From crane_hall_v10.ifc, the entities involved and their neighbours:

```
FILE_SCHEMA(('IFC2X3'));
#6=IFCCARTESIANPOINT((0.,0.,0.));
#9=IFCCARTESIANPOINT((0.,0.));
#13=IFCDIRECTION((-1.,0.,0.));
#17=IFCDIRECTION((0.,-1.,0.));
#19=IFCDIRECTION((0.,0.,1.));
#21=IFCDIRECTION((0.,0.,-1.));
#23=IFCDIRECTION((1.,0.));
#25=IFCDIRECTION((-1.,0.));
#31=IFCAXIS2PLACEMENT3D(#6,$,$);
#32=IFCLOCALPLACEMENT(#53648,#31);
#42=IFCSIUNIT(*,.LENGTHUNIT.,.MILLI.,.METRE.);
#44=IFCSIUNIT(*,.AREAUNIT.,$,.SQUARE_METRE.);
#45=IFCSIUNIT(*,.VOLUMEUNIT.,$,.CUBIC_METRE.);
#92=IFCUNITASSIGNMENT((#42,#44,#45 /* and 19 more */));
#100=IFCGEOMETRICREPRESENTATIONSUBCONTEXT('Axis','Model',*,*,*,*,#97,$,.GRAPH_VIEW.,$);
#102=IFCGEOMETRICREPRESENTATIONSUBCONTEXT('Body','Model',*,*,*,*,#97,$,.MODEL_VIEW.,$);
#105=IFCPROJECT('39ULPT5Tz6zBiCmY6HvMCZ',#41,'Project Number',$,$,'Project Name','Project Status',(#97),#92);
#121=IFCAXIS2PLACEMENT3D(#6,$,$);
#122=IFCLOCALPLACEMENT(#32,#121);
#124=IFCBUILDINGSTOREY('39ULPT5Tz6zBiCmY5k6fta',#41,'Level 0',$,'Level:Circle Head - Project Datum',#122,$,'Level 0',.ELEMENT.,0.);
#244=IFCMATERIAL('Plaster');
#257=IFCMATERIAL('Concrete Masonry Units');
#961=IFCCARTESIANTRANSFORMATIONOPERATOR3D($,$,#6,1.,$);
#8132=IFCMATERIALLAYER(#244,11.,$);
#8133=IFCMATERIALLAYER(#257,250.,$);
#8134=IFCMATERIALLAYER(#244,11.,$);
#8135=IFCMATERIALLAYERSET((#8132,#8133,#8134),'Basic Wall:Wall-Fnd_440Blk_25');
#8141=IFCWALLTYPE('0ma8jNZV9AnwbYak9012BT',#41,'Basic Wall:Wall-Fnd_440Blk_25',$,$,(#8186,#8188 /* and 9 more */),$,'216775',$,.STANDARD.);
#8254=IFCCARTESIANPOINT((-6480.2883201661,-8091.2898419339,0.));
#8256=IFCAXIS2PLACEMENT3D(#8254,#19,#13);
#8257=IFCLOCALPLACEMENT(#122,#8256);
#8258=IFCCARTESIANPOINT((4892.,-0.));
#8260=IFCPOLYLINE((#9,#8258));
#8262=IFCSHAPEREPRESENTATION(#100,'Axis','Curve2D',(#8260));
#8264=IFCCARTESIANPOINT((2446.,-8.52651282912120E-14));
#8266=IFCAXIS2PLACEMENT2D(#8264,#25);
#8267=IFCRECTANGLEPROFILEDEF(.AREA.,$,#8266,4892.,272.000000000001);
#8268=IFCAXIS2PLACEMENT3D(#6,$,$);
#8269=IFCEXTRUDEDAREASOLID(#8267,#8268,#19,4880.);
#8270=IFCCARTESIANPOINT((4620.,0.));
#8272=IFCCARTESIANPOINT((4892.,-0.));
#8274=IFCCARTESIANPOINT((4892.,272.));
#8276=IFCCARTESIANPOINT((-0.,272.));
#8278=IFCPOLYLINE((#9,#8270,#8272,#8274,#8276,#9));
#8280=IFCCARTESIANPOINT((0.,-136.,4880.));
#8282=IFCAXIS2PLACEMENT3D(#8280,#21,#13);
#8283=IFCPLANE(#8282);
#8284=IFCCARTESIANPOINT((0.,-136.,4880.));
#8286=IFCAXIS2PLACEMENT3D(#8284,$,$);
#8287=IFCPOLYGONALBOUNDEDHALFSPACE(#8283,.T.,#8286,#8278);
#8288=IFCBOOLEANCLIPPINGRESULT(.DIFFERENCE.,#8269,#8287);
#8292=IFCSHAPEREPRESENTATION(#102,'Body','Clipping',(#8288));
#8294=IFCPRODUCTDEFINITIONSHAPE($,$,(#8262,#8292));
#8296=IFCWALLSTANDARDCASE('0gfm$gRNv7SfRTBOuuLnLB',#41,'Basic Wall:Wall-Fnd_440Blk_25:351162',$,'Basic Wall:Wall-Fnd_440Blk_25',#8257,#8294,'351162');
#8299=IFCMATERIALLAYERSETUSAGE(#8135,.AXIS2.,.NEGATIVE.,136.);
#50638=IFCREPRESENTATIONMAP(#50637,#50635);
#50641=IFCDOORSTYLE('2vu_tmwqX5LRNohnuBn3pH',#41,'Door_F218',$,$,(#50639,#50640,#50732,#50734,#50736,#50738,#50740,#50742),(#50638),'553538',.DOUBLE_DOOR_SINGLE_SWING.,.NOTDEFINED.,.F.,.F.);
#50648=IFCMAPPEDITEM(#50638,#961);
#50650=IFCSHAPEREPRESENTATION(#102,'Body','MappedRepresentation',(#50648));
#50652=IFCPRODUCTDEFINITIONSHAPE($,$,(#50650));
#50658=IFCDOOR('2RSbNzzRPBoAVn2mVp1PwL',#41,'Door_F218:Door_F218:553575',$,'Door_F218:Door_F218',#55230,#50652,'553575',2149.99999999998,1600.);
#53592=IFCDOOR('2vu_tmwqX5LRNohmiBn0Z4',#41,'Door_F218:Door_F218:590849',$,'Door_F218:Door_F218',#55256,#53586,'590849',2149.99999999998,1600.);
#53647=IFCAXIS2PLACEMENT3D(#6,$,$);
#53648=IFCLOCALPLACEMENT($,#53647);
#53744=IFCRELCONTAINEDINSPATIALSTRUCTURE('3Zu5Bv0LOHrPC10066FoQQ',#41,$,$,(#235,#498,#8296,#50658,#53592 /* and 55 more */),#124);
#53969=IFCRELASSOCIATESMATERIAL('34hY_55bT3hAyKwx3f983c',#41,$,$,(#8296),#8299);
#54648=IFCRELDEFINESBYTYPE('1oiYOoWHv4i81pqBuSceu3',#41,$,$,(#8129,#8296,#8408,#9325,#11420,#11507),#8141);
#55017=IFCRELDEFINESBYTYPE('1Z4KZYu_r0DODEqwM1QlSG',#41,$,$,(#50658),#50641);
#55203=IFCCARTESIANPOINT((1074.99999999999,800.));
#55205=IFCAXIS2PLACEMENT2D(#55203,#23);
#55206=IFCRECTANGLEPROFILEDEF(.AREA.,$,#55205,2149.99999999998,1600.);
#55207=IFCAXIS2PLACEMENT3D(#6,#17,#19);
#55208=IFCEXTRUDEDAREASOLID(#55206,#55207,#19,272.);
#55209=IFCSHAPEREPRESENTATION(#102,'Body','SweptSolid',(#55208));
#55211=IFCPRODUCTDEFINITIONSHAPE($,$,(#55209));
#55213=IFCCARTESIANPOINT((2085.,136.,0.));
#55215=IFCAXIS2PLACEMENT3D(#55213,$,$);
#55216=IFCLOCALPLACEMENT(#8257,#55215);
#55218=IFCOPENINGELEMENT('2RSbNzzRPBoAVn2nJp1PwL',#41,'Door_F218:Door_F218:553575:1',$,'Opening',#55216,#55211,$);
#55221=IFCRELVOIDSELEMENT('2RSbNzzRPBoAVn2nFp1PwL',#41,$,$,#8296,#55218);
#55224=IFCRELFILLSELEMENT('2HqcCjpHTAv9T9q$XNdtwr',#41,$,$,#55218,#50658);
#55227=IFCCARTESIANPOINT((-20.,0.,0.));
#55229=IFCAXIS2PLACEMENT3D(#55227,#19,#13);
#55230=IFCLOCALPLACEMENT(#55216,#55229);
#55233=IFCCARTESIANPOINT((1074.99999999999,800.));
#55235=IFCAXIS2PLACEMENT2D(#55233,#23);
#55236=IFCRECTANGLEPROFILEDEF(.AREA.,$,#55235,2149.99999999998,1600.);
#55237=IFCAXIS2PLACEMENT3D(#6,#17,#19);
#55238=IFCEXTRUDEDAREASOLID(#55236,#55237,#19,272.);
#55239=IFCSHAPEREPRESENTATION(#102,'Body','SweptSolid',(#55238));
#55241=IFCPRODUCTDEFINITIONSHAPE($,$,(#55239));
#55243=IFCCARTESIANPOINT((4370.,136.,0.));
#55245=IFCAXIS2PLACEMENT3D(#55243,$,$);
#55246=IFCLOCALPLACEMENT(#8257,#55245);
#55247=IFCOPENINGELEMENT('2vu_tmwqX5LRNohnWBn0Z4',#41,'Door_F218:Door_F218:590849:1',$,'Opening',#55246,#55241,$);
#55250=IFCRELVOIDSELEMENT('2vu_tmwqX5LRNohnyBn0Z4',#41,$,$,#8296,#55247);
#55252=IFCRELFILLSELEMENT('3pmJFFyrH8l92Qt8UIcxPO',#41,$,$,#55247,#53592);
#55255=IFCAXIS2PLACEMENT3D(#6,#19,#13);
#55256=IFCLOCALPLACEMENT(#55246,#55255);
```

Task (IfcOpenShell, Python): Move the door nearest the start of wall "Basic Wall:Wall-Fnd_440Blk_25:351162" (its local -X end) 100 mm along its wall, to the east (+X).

```python
import ifcopenshell
import ifcopenshell.api.geometry
import ifcopenshell.util.placement
import ifcopenshell.util.unit

model = ifcopenshell.open("crane_hall_v10.ifc")
unit_scale = ifcopenshell.util.unit.calculate_unit_scale(model)

door = model.by_guid("2RSbNzzRPBoAVn2mVp1PwL")
opening = door.FillsVoids[0].RelatingOpeningElement
wall = opening.VoidsElements[0].RelatingBuildingElement

wall_matrix = ifcopenshell.util.placement.get_local_placement(wall.ObjectPlacement)
shift = wall_matrix[:3, 0] * -0.1 / unit_scale
before = ifcopenshell.util.placement.get_local_placement(door.ObjectPlacement)[:3, 3].copy()

# The door is placed relative to its opening, so it follows when the opening moves.
matrix = ifcopenshell.util.placement.get_local_placement(opening.ObjectPlacement)
matrix[:3, 3] += shift
ifcopenshell.api.geometry.edit_object_placement(
    model, product=opening, matrix=matrix, is_si=False, should_transform_children=True
)

after = ifcopenshell.util.placement.get_local_placement(door.ObjectPlacement)[:3, 3]
print("door moved by", (after - before).round(3) + 0.0)

model.write("crane_hall_v10_edited.ifc")
```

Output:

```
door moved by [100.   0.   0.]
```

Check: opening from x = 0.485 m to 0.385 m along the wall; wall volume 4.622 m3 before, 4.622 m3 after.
